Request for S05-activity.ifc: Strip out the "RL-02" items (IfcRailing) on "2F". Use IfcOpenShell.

First a look at what the model holds.

```python
import ifcopenshell
import ifcopenshell.util.element

model = ifcopenshell.open("S05-activity.ifc")
print(model.schema)
storey = next(s for s in model.by_type("IfcBuildingStorey") if s.Name == "2F")
railings = [e for e in ifcopenshell.util.element.get_decomposition(storey) if e.is_a("IfcRailing")]
seen = {}
for e in railings:
    element_type = ifcopenshell.util.element.get_type(e)
    name = element_type.Name if element_type not in (None, e) else None
    seen[name] = seen.get(name, 0) + 1
for name, count in sorted(seen.items(), key=str):
    print(count, "x", name)
```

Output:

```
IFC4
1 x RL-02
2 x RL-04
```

```python
import ifcopenshell
import ifcopenshell.api.root
import ifcopenshell.util.element

model = ifcopenshell.open("S05-activity.ifc")

storey = next(s for s in model.by_type("IfcBuildingStorey") if s.Name == "2F")
railings = [e for e in ifcopenshell.util.element.get_decomposition(storey) if e.is_a("IfcRailing")]
targets = [e for e in railings if (t := ifcopenshell.util.element.get_type(e)) not in (None, e) and t.Name == "RL-02"]

for e in targets:
    ifcopenshell.api.root.remove_product(model, product=e)
print(len(targets), "removed")

model.write("S05-activity_edited.ifc")
```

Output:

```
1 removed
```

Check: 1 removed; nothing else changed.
